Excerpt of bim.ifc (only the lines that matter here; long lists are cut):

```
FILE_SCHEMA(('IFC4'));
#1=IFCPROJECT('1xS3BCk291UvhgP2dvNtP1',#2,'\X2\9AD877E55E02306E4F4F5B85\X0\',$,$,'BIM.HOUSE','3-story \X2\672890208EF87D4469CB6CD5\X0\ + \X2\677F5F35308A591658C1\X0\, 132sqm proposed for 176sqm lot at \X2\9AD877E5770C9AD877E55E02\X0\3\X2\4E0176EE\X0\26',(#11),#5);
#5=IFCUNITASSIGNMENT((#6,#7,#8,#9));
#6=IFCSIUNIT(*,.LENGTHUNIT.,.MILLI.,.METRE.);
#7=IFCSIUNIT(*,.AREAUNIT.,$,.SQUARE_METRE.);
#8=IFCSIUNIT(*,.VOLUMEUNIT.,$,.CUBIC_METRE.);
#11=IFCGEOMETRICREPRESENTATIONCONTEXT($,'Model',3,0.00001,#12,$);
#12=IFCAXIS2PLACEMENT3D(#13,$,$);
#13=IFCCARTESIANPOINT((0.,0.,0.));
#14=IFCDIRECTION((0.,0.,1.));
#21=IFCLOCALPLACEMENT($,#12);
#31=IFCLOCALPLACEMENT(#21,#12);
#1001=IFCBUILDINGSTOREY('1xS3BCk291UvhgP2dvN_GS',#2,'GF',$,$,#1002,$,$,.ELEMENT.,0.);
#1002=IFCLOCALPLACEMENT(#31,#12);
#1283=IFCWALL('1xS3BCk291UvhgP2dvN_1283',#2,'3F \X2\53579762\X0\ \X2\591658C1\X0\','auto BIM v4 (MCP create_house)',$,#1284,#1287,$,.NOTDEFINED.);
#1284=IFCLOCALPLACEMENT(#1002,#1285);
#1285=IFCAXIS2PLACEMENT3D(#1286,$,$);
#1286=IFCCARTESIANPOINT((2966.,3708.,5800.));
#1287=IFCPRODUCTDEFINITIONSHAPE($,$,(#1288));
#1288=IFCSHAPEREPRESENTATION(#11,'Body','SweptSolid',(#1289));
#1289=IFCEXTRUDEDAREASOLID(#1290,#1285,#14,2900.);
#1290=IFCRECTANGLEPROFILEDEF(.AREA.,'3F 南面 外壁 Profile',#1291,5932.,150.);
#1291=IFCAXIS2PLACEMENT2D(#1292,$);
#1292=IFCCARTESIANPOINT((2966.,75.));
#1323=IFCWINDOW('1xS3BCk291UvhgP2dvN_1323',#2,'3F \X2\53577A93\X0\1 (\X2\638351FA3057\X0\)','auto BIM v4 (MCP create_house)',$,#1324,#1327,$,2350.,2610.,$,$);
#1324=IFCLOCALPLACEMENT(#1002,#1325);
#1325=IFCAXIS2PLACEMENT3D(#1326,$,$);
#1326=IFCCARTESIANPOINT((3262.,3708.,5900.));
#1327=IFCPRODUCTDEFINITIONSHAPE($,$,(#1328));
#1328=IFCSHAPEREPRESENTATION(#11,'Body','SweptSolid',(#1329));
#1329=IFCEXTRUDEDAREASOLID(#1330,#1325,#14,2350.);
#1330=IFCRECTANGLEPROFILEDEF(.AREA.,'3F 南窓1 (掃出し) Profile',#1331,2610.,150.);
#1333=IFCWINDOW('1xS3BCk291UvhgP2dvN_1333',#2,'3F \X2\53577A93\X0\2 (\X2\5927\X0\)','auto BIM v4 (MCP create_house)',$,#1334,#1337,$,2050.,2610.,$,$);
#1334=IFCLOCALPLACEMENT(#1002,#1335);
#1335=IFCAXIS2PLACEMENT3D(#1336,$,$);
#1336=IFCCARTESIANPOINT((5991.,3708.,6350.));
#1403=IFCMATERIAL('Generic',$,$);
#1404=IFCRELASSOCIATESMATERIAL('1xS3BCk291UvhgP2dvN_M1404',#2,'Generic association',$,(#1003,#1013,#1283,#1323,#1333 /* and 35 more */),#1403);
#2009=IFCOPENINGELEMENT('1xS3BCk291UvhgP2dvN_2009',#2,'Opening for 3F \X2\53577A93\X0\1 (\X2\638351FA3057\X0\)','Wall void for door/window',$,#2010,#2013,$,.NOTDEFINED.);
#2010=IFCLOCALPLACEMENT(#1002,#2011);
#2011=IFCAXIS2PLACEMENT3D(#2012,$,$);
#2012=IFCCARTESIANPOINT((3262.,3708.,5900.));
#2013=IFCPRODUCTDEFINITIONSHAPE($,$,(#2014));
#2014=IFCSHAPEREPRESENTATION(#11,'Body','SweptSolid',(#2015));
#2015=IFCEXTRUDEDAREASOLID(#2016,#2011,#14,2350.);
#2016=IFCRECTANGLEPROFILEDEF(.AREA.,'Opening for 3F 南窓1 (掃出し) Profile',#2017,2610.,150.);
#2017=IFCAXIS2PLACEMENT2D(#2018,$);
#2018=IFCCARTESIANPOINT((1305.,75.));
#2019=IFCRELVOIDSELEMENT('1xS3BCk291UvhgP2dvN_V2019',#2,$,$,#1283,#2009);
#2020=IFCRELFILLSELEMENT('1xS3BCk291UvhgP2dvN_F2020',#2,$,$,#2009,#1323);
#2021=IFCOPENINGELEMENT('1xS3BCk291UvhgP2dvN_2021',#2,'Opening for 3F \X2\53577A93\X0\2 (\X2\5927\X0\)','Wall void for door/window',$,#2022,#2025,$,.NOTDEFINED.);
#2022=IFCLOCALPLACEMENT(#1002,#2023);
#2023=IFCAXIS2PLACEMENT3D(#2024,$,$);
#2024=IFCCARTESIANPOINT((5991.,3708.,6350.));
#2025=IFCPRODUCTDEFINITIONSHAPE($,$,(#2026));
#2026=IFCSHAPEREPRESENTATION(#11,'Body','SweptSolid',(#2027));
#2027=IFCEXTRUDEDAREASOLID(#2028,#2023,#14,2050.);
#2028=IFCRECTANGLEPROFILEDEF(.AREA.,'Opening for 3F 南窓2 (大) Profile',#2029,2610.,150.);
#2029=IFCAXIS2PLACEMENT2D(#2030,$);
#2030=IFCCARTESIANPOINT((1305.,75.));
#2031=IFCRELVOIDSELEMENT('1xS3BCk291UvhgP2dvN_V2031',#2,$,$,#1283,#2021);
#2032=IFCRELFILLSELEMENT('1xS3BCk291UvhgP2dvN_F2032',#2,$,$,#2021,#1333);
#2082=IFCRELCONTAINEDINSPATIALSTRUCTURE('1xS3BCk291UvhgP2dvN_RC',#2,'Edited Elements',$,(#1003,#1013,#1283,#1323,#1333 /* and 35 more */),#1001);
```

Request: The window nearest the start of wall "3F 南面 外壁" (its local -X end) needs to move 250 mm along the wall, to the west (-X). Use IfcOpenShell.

```python
import ifcopenshell
import ifcopenshell.api.geometry
import ifcopenshell.util.placement
import ifcopenshell.util.unit

model = ifcopenshell.open("bim.ifc")
unit_scale = ifcopenshell.util.unit.calculate_unit_scale(model)

window = model.by_id(1323)
opening = window.FillsVoids[0].RelatingOpeningElement
wall = opening.VoidsElements[0].RelatingBuildingElement

wall_matrix = ifcopenshell.util.placement.get_local_placement(wall.ObjectPlacement)
shift = wall_matrix[:3, 0] * -0.25 / unit_scale
before = ifcopenshell.util.placement.get_local_placement(window.ObjectPlacement)[:3, 3].copy()

# The window is not placed relative to its opening, so move both.
for product in (opening, window):
    matrix = ifcopenshell.util.placement.get_local_placement(product.ObjectPlacement)
    matrix[:3, 3] += shift
    ifcopenshell.api.geometry.edit_object_placement(model, product=product, matrix=matrix, is_si=False)

after = ifcopenshell.util.placement.get_local_placement(window.ObjectPlacement)[:3, 3]
print("window moved by", (after - before).round(3) + 0.0)

model.write("bim-out.ifc")
```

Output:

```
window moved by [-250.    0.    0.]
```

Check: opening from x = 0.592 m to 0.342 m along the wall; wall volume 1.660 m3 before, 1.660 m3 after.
